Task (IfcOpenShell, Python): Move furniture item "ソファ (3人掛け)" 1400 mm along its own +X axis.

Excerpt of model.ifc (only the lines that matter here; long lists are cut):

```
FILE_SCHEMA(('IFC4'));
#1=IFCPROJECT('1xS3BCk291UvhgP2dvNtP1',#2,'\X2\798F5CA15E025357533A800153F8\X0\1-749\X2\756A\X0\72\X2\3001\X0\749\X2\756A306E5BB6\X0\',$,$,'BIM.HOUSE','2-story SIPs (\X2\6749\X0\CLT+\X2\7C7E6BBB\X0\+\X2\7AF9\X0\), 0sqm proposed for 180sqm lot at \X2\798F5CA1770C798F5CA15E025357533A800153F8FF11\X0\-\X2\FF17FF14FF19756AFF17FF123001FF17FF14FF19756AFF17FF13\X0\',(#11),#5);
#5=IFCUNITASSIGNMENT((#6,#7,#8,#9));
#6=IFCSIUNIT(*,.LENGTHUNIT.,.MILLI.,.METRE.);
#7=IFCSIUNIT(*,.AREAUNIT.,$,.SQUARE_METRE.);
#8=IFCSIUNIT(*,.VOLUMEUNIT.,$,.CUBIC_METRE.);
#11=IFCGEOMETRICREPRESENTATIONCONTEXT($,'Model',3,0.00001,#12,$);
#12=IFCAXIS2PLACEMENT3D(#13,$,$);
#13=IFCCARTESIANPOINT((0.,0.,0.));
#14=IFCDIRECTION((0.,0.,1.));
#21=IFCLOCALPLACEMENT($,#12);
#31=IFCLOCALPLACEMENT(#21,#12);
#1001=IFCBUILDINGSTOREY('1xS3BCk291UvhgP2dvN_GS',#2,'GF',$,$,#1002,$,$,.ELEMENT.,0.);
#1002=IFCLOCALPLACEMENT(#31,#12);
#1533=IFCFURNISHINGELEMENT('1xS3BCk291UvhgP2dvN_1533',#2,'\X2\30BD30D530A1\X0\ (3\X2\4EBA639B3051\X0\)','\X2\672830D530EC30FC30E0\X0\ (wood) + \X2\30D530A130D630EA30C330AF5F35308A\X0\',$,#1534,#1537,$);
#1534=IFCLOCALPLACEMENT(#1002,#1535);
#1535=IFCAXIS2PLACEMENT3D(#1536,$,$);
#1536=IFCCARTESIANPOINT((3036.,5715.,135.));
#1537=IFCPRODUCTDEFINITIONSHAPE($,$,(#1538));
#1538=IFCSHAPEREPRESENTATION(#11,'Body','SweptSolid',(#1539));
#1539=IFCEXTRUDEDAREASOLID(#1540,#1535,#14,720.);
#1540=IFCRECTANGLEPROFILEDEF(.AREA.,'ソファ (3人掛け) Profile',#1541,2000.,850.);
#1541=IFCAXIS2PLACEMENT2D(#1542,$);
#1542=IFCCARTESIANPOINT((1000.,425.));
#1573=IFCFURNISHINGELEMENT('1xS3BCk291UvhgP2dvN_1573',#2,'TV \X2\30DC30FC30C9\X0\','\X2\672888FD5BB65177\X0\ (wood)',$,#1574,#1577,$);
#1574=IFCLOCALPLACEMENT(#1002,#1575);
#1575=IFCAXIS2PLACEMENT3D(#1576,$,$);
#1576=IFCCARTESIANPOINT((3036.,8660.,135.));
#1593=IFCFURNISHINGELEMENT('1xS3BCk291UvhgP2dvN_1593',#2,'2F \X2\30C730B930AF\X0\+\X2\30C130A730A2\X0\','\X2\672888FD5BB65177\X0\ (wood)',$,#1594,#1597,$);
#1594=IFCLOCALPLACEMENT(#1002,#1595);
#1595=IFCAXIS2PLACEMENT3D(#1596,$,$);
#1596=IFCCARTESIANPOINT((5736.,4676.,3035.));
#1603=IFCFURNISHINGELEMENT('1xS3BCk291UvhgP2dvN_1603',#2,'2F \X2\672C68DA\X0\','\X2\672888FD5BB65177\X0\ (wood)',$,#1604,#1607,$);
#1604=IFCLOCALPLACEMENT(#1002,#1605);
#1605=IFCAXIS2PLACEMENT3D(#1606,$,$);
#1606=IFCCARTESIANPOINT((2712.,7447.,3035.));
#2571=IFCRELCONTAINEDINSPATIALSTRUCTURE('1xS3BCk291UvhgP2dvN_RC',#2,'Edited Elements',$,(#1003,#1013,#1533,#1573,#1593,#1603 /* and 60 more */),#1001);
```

```python
import ifcopenshell
import ifcopenshell.api.geometry
import ifcopenshell.util.placement
import ifcopenshell.util.unit

model = ifcopenshell.open("model.ifc")
unit_scale = ifcopenshell.util.unit.calculate_unit_scale(model)

item = model.by_guid("1xS3BCk291UvhgP2dvN_1533")
matrix = ifcopenshell.util.placement.get_local_placement(item.ObjectPlacement)
matrix[:3, 3] += matrix[:3, 0] * 1.4 / unit_scale
ifcopenshell.api.geometry.edit_object_placement(model, product=item, matrix=matrix, is_si=False)

print(ifcopenshell.util.placement.get_local_placement(item.ObjectPlacement).round(3) + 0.0)

model.write("model_edited.ifc")
```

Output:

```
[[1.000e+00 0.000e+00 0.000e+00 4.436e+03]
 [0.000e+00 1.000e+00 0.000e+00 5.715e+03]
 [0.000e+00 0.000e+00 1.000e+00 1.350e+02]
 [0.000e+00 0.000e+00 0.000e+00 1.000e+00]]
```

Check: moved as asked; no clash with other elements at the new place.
